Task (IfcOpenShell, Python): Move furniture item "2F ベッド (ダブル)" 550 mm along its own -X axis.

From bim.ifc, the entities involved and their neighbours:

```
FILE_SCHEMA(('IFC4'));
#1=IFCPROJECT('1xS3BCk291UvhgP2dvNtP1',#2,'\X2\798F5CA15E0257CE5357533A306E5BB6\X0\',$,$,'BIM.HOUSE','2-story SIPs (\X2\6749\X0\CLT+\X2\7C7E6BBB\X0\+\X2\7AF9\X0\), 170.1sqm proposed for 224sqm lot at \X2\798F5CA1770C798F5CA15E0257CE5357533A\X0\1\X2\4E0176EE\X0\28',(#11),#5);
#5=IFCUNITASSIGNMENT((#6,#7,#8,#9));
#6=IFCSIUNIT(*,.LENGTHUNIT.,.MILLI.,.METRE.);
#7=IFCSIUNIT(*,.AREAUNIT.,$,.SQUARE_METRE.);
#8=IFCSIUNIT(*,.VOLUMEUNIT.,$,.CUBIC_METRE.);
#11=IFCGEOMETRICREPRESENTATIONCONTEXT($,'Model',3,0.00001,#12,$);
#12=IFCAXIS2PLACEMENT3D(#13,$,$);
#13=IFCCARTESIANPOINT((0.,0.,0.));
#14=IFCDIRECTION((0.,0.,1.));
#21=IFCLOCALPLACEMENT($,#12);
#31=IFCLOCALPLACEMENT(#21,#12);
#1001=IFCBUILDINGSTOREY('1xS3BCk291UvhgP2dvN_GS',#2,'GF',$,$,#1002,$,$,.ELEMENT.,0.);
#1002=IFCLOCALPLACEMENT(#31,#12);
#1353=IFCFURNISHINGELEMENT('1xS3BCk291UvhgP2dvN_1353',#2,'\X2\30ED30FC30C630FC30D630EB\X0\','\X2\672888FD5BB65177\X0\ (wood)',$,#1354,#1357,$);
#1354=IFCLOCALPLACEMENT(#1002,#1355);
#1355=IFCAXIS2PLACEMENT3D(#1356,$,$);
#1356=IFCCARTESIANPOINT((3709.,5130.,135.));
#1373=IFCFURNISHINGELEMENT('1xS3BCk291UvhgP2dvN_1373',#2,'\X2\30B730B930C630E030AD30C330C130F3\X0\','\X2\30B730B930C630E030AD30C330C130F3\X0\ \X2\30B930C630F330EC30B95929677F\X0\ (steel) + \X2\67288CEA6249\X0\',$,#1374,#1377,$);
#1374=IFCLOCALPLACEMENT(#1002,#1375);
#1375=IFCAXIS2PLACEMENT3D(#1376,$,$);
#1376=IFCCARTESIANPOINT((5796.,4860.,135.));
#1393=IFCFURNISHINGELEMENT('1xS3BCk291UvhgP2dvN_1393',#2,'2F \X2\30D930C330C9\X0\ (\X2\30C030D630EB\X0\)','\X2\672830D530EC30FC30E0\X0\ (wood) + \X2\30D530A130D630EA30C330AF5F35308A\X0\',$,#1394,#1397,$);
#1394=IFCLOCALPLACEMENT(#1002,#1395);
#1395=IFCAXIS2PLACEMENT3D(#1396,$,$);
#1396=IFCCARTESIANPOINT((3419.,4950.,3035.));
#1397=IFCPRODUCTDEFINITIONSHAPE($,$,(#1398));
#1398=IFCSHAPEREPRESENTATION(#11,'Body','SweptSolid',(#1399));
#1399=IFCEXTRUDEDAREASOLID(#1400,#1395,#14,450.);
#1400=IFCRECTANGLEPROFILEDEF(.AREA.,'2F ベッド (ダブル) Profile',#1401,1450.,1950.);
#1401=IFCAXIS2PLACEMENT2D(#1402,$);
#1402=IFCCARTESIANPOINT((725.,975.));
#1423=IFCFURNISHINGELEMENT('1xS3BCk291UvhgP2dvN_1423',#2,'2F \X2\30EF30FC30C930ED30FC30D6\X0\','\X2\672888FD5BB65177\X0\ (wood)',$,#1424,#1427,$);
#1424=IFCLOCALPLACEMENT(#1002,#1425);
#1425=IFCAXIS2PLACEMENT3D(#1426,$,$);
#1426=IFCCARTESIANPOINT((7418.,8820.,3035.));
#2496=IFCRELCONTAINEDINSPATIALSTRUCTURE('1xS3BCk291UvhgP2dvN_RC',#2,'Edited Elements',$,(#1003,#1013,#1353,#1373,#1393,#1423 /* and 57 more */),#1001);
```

```python
import ifcopenshell
import ifcopenshell.api.geometry
import ifcopenshell.util.placement
import ifcopenshell.util.unit

model = ifcopenshell.open("bim.ifc")
unit_scale = ifcopenshell.util.unit.calculate_unit_scale(model)

item = model.by_guid("1xS3BCk291UvhgP2dvN_1393")
matrix = ifcopenshell.util.placement.get_local_placement(item.ObjectPlacement)
matrix[:3, 3] -= matrix[:3, 0] * 0.55 / unit_scale
ifcopenshell.api.geometry.edit_object_placement(model, product=item, matrix=matrix, is_si=False)

print(ifcopenshell.util.placement.get_local_placement(item.ObjectPlacement).round(3) + 0.0)

model.write("bim_updated.ifc")
```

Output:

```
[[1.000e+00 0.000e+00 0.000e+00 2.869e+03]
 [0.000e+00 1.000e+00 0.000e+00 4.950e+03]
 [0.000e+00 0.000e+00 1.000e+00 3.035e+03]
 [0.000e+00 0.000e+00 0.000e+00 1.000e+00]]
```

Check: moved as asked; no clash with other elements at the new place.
